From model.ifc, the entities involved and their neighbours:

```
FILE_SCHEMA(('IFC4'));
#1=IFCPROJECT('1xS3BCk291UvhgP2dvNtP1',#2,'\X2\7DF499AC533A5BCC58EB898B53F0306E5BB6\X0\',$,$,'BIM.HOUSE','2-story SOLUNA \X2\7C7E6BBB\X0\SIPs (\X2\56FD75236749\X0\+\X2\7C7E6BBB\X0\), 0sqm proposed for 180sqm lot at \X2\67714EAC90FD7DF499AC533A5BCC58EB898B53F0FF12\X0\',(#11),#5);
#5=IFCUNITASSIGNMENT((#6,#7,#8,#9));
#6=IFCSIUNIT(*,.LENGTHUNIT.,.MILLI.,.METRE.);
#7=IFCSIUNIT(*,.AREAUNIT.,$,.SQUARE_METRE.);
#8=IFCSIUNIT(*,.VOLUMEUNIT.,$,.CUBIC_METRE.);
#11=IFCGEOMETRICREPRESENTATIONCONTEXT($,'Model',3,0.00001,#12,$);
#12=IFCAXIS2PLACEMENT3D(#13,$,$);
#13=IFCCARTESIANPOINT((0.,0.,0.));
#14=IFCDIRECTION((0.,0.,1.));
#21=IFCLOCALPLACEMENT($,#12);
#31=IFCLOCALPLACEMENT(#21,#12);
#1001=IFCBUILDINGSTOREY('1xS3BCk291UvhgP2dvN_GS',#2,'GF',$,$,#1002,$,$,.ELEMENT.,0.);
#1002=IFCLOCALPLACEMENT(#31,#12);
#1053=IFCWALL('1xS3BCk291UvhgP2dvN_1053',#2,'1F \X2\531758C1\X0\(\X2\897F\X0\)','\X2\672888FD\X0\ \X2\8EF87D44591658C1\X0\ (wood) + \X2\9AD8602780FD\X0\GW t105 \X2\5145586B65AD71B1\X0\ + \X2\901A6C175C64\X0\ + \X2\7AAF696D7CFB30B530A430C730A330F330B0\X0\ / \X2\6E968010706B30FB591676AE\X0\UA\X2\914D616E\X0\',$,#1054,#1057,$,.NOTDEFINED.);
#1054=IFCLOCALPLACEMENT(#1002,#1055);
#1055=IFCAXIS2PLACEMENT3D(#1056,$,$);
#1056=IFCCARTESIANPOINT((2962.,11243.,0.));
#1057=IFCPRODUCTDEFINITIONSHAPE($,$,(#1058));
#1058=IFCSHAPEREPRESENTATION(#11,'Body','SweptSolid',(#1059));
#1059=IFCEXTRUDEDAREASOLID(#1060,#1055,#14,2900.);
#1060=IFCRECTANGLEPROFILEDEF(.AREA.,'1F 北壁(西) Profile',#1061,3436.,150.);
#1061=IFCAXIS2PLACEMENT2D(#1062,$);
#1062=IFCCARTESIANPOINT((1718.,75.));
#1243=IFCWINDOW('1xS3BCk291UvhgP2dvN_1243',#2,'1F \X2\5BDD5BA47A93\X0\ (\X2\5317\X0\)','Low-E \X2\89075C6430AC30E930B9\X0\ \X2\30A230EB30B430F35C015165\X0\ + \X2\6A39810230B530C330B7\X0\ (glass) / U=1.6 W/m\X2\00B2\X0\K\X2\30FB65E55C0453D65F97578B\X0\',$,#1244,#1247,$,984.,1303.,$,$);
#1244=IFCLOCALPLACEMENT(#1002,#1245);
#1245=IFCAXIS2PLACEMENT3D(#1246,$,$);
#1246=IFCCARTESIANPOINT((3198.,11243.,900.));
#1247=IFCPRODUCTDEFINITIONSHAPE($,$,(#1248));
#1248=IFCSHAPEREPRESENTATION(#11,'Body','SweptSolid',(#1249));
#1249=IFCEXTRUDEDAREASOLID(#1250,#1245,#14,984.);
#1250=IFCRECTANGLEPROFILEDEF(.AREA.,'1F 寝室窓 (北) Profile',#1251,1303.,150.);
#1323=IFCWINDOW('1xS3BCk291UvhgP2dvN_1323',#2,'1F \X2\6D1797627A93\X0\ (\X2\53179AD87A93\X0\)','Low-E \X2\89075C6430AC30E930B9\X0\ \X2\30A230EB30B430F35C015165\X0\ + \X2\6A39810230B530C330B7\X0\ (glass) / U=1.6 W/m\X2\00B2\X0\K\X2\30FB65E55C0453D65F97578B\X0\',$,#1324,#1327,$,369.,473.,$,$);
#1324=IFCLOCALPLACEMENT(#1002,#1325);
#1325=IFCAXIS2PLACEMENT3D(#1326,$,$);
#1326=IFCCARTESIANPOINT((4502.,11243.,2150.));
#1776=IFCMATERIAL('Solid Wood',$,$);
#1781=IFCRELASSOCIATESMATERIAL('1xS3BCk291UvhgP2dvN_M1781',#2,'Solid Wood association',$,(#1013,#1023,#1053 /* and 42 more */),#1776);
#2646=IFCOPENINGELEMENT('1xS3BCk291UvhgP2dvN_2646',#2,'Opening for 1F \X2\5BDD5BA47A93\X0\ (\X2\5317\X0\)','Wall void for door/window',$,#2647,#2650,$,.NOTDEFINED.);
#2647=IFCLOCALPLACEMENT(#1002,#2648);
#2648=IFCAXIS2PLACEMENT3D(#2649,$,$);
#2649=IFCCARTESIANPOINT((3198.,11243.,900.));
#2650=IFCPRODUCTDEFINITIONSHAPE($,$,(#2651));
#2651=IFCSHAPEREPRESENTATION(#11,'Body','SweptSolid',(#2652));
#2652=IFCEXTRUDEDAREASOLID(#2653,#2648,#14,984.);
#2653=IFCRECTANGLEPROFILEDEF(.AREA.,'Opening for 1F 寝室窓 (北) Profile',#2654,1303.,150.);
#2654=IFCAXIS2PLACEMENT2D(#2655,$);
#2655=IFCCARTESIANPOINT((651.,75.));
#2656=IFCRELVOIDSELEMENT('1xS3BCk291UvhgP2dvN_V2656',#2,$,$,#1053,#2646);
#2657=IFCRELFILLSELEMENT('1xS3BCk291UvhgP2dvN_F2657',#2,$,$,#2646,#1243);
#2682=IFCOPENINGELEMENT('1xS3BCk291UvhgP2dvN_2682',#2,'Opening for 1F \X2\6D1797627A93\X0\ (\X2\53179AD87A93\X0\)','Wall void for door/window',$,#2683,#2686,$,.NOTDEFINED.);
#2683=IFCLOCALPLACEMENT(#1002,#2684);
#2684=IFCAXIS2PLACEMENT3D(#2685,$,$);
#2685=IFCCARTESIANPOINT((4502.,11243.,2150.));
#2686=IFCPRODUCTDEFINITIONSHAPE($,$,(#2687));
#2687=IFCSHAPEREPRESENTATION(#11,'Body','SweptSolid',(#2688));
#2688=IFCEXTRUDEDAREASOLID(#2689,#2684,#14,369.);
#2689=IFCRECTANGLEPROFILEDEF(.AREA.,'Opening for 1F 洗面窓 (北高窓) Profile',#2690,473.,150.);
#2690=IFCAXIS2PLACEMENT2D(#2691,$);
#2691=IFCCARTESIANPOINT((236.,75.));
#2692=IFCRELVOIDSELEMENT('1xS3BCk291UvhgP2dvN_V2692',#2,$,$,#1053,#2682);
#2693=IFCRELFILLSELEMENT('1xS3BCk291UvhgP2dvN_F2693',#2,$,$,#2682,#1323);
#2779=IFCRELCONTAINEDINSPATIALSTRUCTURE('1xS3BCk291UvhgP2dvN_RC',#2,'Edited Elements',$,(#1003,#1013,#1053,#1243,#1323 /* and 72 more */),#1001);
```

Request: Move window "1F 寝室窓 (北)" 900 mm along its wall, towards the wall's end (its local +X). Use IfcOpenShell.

```python
import ifcopenshell
import ifcopenshell.api.geometry
import ifcopenshell.util.placement
import ifcopenshell.util.unit

model = ifcopenshell.open("model.ifc")
unit_scale = ifcopenshell.util.unit.calculate_unit_scale(model)

window = model.by_guid("1xS3BCk291UvhgP2dvN_1243")
opening = window.FillsVoids[0].RelatingOpeningElement
wall = opening.VoidsElements[0].RelatingBuildingElement

wall_matrix = ifcopenshell.util.placement.get_local_placement(wall.ObjectPlacement)
shift = wall_matrix[:3, 0] * 0.9 / unit_scale
before = ifcopenshell.util.placement.get_local_placement(window.ObjectPlacement)[:3, 3].copy()

# The window is not placed relative to its opening, so move both.
for product in (opening, window):
    matrix = ifcopenshell.util.placement.get_local_placement(product.ObjectPlacement)
    matrix[:3, 3] += shift
    ifcopenshell.api.geometry.edit_object_placement(model, product=product, matrix=matrix, is_si=False)

after = ifcopenshell.util.placement.get_local_placement(window.ObjectPlacement)[:3, 3]
print("window moved by", (after - before).round(3) + 0.0)

model.write("model_edited.ifc")
```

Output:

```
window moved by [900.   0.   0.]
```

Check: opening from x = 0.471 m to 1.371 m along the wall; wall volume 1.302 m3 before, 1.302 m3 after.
